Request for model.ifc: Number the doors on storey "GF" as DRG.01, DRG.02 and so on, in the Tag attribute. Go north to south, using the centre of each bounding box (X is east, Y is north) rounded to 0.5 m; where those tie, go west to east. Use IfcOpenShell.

First a look at what the model holds.

```python
import ifcopenshell
import ifcopenshell.util.element
import ifcopenshell.util.placement

model = ifcopenshell.open("model.ifc")
print(model.schema)
storey = next(s for s in model.by_type("IfcBuildingStorey") if s.Name == "GF")
doors = [e for e in ifcopenshell.util.element.get_decomposition(storey) if e.is_a("IfcDoor")]
for e in sorted(doors, key=lambda e: e.id()):
    origin = ifcopenshell.util.placement.get_local_placement(e.ObjectPlacement)[:3, 3]
    print(e.id(), e.Tag, e.Name, origin.round(2) + 0.0, sep=" | ")
```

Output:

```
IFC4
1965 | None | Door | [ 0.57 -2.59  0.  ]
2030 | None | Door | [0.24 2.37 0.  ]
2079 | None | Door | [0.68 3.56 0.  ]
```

```python
import ifcopenshell
import ifcopenshell.geom
import ifcopenshell.util.element
import ifcopenshell.util.shape

model = ifcopenshell.open("model.ifc")
settings = ifcopenshell.geom.settings()
settings.set("use-world-coords", True)


def centre(element):
    shape = ifcopenshell.geom.create_shape(settings, element)
    return ifcopenshell.util.shape.get_bbox_centroid(shape.geometry)


storey = next(s for s in model.by_type("IfcBuildingStorey") if s.Name == "GF")
doors = [e for e in ifcopenshell.util.element.get_decomposition(storey) if e.is_a("IfcDoor")]

# Insertion points can sit at a corner or the storey origin, so sort by the geometry (in metres).
centres = {e: centre(e) for e in doors}
doors.sort(key=lambda e: (-round(centres[e][1] / 0.5), centres[e][0]))

for i, e in enumerate(doors, start=1):
    number = f"DRG.{i:02d}"
    e.Tag = number
    print(e.id(), number)

model.write("model_rev.ifc")
```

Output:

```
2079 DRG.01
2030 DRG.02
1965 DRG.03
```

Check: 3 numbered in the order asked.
